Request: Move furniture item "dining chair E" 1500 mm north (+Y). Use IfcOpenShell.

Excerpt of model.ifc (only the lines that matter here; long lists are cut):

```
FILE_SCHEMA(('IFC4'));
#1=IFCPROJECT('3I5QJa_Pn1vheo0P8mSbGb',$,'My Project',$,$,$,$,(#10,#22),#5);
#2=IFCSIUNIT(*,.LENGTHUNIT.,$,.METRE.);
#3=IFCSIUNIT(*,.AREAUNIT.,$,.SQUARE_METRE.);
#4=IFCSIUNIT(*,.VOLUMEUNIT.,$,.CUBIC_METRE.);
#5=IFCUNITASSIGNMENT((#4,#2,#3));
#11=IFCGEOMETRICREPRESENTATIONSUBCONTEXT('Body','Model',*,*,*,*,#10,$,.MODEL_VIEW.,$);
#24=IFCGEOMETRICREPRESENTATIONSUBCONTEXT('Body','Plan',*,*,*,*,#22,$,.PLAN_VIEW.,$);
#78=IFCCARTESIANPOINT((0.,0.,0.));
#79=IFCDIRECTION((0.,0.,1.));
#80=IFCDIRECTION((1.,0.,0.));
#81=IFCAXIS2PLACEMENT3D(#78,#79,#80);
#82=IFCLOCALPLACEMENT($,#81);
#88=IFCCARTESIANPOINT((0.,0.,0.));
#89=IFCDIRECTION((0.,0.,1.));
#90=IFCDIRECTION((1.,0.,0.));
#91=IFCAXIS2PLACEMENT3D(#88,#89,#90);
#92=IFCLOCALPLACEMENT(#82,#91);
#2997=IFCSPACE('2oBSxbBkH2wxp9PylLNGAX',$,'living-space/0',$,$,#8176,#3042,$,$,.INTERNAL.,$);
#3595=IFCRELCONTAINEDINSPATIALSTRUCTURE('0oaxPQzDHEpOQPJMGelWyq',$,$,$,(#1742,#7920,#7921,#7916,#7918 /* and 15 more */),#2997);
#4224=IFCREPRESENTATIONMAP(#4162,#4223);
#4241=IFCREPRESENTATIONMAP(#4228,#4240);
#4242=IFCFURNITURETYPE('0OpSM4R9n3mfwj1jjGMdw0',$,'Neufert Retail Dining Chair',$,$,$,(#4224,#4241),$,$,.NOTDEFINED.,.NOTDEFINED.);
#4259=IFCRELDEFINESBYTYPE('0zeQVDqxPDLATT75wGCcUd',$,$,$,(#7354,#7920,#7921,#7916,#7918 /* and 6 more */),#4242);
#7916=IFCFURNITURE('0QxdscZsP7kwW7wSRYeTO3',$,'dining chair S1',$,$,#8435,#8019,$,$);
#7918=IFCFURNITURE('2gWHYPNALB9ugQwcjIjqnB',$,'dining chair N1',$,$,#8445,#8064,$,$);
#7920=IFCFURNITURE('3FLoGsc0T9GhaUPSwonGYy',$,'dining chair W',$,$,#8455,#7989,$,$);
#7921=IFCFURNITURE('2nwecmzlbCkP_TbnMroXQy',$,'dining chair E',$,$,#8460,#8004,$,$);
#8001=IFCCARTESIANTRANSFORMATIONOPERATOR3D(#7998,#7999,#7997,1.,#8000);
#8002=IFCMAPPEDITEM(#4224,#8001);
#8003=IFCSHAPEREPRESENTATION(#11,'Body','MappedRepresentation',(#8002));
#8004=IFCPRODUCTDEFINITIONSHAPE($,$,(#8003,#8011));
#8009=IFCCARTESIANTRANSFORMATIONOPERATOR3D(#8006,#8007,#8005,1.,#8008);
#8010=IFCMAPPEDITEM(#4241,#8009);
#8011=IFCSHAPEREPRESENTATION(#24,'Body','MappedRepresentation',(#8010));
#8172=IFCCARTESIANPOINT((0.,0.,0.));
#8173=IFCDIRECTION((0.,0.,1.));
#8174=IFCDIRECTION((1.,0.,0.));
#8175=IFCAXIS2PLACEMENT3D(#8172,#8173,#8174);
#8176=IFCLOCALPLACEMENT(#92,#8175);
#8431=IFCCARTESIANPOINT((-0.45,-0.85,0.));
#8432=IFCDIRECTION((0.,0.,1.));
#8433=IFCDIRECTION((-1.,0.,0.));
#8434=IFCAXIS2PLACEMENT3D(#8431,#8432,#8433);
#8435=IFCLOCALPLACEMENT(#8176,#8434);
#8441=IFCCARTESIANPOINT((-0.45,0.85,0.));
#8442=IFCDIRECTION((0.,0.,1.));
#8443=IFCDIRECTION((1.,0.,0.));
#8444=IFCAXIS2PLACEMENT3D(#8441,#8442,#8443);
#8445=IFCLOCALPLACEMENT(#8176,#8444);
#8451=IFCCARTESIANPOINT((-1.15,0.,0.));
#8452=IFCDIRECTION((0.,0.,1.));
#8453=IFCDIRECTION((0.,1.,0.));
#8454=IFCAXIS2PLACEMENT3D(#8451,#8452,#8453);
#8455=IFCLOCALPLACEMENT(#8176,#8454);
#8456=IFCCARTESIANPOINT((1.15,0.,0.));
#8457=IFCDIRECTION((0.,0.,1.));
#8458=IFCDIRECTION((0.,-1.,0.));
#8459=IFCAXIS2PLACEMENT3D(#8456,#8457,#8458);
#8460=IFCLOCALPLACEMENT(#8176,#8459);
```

```python
import ifcopenshell
import ifcopenshell.api.geometry
import ifcopenshell.util.placement
import ifcopenshell.util.unit

model = ifcopenshell.open("model.ifc")
unit_scale = ifcopenshell.util.unit.calculate_unit_scale(model)

item = model.by_guid("2nwecmzlbCkP_TbnMroXQy")
matrix = ifcopenshell.util.placement.get_local_placement(item.ObjectPlacement)
matrix[1, 3] += 1.5 / unit_scale
ifcopenshell.api.geometry.edit_object_placement(model, product=item, matrix=matrix, is_si=False)

print(ifcopenshell.util.placement.get_local_placement(item.ObjectPlacement).round(3) + 0.0)

model.write("model_edited.ifc")
```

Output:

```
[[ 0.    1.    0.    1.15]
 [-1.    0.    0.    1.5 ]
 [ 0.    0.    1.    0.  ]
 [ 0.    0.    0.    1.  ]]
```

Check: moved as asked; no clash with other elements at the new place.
